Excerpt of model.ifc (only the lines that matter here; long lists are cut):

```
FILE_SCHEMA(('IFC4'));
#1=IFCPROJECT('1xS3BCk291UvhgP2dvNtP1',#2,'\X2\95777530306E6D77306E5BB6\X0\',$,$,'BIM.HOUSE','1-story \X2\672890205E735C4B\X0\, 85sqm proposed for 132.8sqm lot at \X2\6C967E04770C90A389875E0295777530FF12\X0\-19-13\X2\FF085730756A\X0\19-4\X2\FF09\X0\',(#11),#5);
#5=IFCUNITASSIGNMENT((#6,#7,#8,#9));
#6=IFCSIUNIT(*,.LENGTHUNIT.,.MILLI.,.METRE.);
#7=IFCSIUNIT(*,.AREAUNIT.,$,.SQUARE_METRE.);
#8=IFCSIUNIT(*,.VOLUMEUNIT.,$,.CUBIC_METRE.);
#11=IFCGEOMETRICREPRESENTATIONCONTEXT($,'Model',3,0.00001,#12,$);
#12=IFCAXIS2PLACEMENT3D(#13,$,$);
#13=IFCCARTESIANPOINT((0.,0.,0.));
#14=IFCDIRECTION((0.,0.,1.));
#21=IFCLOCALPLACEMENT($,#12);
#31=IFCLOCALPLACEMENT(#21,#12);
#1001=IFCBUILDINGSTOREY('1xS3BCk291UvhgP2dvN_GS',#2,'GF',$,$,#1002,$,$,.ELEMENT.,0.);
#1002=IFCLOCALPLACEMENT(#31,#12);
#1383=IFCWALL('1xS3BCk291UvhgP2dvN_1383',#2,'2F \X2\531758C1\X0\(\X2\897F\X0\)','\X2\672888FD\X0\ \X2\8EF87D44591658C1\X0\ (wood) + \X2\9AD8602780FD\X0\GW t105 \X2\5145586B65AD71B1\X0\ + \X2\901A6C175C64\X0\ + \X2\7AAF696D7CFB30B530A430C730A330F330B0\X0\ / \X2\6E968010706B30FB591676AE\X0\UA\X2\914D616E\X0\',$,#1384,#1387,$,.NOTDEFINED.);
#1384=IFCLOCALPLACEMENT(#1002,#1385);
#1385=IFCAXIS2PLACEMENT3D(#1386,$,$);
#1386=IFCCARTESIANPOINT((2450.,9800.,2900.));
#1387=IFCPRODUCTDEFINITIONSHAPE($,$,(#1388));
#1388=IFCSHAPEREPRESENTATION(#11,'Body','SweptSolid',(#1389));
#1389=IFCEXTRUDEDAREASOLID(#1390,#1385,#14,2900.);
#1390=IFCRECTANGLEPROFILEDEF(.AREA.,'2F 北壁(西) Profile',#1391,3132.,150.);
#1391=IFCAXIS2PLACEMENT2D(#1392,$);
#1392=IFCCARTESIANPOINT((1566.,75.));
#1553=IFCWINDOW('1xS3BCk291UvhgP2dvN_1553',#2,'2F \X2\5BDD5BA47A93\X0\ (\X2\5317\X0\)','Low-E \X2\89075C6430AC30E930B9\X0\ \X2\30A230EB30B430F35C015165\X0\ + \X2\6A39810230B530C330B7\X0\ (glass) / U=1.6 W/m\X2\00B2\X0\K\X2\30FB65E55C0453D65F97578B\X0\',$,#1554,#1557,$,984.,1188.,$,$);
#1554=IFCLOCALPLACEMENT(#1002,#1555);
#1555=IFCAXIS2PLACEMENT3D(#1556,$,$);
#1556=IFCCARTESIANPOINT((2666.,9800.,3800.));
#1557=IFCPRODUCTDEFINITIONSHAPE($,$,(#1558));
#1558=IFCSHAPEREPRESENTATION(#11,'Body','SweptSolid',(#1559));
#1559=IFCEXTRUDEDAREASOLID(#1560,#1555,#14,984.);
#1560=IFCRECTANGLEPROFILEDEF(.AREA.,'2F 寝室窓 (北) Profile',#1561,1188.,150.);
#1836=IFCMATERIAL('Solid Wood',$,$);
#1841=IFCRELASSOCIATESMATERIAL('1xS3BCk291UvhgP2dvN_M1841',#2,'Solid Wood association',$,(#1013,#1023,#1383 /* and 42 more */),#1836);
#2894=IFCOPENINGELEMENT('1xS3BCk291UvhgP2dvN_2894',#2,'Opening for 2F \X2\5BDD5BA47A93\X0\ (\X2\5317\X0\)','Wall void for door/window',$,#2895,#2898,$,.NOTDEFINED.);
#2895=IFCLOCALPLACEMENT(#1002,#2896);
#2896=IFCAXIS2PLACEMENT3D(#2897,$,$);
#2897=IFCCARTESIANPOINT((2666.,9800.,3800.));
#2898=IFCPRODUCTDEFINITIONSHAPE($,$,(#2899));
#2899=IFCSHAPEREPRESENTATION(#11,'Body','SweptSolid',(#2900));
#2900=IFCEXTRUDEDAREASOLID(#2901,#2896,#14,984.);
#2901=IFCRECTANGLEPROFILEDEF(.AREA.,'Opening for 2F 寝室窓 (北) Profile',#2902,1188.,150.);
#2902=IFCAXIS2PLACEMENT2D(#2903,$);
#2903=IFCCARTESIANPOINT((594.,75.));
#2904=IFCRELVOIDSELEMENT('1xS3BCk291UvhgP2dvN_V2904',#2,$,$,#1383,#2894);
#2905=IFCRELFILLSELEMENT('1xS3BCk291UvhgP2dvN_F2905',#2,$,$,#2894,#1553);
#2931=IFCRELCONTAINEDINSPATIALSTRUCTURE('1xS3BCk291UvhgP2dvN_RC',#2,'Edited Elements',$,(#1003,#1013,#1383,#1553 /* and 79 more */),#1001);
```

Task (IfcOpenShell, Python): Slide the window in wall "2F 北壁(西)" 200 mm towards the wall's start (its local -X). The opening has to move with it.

```python
import ifcopenshell
import ifcopenshell.api.geometry
import ifcopenshell.util.placement

model = ifcopenshell.open("model.ifc")

window = model.by_guid("1xS3BCk291UvhgP2dvN_1553")
opening = window.FillsVoids[0].RelatingOpeningElement
wall = opening.VoidsElements[0].RelatingBuildingElement

wall_matrix = ifcopenshell.util.placement.get_local_placement(wall.ObjectPlacement)
shift = wall_matrix[:3, 0] * -200.0
before = ifcopenshell.util.placement.get_local_placement(window.ObjectPlacement)[:3, 3].copy()

# The window is not placed relative to its opening, so move both.
for product in (opening, window):
    matrix = ifcopenshell.util.placement.get_local_placement(product.ObjectPlacement)
    matrix[:3, 3] += shift
    ifcopenshell.api.geometry.edit_object_placement(model, product=product, matrix=matrix, is_si=False)

after = ifcopenshell.util.placement.get_local_placement(window.ObjectPlacement)[:3, 3]
print("window moved by", (after - before).round(3) + 0.0)

model.write("model_updated.ifc")
```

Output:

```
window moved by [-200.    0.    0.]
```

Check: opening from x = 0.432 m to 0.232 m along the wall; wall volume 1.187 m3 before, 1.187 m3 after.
